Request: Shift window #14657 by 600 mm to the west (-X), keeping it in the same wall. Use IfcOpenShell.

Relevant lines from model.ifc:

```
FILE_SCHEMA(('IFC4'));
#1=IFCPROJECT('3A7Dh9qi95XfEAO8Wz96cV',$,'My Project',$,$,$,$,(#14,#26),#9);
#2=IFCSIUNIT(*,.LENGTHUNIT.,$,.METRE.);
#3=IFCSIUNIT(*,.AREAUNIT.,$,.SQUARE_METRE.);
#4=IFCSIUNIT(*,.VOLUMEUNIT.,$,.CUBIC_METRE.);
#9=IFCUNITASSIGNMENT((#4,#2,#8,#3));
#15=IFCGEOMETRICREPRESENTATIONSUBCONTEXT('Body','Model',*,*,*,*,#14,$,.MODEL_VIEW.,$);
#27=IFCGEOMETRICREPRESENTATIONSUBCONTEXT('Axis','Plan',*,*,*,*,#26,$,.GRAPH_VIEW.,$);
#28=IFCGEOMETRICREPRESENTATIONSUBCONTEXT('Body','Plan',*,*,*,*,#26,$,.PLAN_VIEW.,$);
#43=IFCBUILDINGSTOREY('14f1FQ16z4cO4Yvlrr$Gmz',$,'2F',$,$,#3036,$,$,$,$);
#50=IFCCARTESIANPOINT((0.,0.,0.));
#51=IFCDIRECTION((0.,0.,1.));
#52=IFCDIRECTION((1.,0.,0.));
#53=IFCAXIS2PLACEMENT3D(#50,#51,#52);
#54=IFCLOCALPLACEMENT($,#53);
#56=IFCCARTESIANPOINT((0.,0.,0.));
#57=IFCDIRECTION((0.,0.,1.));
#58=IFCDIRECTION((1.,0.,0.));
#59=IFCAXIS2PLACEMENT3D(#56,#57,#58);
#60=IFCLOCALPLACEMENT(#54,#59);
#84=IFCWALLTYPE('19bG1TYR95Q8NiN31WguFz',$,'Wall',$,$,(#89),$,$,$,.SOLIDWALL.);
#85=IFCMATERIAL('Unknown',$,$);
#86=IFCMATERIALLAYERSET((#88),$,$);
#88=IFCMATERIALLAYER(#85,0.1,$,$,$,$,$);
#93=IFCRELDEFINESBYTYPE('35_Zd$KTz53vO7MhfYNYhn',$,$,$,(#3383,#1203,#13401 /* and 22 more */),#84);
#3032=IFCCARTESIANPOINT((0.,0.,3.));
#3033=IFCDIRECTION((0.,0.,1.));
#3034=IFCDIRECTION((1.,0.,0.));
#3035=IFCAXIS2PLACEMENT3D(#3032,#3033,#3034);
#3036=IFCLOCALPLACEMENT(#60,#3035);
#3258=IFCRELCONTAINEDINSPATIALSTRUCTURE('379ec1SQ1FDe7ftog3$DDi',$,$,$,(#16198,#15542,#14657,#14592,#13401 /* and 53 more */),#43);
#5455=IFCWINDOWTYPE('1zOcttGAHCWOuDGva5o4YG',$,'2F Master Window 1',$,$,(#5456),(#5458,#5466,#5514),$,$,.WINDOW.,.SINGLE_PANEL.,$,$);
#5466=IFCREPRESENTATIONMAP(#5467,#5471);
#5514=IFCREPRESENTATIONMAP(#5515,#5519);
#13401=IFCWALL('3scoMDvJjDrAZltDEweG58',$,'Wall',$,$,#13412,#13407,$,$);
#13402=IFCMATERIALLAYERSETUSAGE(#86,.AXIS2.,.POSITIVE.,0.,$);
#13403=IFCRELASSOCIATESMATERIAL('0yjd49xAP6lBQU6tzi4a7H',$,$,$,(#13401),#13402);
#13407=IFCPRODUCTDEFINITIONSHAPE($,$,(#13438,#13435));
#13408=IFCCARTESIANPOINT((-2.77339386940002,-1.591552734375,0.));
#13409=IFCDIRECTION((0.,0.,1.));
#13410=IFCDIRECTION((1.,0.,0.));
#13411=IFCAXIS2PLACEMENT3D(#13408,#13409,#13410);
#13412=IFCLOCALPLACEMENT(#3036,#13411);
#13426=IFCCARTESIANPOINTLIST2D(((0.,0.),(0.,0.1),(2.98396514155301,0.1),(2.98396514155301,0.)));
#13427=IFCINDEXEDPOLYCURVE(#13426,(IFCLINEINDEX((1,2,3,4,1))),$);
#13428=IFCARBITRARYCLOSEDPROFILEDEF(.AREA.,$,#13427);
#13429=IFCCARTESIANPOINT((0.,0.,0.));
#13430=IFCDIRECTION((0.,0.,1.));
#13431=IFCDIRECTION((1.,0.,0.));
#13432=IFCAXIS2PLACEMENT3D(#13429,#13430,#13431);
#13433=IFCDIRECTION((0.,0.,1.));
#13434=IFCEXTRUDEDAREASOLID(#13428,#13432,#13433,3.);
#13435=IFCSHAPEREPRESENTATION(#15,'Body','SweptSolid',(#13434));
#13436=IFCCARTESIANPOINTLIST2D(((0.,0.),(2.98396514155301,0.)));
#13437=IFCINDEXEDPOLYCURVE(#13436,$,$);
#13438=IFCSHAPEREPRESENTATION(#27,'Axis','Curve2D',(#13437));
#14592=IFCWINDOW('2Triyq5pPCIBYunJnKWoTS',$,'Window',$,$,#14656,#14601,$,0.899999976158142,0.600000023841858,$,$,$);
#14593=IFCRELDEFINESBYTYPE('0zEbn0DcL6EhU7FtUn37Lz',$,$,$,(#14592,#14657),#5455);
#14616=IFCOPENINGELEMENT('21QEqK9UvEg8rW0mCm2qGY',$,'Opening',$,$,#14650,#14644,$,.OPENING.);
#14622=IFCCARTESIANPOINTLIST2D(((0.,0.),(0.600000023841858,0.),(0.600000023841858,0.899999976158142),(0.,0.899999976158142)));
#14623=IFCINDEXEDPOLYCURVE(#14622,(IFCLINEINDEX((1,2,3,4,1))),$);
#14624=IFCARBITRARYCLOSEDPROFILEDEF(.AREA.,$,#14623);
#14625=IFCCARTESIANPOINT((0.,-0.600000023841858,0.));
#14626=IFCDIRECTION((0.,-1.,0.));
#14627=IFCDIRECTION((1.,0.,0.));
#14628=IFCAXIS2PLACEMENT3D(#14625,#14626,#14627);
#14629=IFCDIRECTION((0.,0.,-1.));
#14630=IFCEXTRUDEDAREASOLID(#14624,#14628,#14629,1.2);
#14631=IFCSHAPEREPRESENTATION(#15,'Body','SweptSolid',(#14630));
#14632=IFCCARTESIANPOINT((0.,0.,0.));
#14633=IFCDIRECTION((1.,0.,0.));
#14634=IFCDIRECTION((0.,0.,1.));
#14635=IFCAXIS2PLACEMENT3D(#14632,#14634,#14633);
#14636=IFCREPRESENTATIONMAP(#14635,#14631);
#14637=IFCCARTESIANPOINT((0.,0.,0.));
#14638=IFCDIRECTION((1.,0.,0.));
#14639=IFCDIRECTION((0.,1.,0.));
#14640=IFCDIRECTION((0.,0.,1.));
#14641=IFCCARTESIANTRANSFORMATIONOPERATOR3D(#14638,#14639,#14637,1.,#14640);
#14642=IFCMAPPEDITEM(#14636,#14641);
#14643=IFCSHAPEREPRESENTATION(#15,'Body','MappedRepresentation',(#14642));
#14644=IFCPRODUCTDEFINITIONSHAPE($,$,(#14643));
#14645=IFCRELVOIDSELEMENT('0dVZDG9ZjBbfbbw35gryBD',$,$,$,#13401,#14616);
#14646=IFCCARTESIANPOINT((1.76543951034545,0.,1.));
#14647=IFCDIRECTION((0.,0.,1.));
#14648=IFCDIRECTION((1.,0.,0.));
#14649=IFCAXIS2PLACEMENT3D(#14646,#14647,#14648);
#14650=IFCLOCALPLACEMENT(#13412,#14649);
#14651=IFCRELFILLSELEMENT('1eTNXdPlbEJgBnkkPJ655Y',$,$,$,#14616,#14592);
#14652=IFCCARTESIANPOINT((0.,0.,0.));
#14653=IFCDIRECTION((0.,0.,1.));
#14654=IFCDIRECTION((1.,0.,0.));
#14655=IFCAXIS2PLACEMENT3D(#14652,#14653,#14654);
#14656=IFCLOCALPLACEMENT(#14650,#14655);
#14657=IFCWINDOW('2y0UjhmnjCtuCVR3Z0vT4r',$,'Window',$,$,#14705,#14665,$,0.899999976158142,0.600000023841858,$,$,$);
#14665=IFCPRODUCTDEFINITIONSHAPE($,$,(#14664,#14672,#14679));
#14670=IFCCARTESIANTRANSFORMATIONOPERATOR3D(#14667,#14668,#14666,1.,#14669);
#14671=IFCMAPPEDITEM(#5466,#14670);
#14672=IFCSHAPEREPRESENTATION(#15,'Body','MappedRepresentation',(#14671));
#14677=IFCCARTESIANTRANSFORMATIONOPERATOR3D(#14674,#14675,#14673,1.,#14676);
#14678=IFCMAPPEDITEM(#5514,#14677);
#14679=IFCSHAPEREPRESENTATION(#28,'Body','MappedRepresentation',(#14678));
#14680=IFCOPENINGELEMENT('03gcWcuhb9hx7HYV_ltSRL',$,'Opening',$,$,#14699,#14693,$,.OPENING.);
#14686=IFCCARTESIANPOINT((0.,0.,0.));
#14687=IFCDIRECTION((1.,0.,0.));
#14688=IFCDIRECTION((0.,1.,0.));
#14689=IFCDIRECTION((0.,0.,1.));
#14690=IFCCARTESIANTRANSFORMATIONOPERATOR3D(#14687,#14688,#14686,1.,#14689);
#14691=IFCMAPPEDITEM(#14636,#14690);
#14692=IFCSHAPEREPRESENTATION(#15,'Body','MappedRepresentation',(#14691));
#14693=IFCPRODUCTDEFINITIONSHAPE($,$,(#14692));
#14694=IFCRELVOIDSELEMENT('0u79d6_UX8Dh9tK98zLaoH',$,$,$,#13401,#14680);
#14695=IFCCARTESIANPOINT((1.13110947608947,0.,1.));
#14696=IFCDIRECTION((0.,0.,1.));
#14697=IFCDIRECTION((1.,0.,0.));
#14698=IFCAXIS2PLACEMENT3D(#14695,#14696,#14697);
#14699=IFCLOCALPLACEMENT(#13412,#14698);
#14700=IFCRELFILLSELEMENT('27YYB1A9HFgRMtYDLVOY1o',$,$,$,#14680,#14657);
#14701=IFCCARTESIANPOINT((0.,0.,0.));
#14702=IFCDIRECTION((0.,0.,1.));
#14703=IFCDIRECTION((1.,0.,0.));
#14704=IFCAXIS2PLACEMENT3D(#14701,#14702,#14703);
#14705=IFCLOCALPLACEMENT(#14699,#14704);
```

```python
import ifcopenshell
import ifcopenshell.api.geometry
import ifcopenshell.util.placement
import ifcopenshell.util.unit

model = ifcopenshell.open("model.ifc")
unit_scale = ifcopenshell.util.unit.calculate_unit_scale(model)

window = model.by_guid("2y0UjhmnjCtuCVR3Z0vT4r")
opening = window.FillsVoids[0].RelatingOpeningElement
wall = opening.VoidsElements[0].RelatingBuildingElement

wall_matrix = ifcopenshell.util.placement.get_local_placement(wall.ObjectPlacement)
shift = wall_matrix[:3, 0] * -0.6 / unit_scale
before = ifcopenshell.util.placement.get_local_placement(window.ObjectPlacement)[:3, 3].copy()

# The window is placed relative to its opening, so it follows when the opening moves.
matrix = ifcopenshell.util.placement.get_local_placement(opening.ObjectPlacement)
matrix[:3, 3] += shift
ifcopenshell.api.geometry.edit_object_placement(
    model, product=opening, matrix=matrix, is_si=False, should_transform_children=True
)

after = ifcopenshell.util.placement.get_local_placement(window.ObjectPlacement)[:3, 3]
print("window moved by", (after - before).round(3) + 0.0)

model.write("model-out.ifc")
```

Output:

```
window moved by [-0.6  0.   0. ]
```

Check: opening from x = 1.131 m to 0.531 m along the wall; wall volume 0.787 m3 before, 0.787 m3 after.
